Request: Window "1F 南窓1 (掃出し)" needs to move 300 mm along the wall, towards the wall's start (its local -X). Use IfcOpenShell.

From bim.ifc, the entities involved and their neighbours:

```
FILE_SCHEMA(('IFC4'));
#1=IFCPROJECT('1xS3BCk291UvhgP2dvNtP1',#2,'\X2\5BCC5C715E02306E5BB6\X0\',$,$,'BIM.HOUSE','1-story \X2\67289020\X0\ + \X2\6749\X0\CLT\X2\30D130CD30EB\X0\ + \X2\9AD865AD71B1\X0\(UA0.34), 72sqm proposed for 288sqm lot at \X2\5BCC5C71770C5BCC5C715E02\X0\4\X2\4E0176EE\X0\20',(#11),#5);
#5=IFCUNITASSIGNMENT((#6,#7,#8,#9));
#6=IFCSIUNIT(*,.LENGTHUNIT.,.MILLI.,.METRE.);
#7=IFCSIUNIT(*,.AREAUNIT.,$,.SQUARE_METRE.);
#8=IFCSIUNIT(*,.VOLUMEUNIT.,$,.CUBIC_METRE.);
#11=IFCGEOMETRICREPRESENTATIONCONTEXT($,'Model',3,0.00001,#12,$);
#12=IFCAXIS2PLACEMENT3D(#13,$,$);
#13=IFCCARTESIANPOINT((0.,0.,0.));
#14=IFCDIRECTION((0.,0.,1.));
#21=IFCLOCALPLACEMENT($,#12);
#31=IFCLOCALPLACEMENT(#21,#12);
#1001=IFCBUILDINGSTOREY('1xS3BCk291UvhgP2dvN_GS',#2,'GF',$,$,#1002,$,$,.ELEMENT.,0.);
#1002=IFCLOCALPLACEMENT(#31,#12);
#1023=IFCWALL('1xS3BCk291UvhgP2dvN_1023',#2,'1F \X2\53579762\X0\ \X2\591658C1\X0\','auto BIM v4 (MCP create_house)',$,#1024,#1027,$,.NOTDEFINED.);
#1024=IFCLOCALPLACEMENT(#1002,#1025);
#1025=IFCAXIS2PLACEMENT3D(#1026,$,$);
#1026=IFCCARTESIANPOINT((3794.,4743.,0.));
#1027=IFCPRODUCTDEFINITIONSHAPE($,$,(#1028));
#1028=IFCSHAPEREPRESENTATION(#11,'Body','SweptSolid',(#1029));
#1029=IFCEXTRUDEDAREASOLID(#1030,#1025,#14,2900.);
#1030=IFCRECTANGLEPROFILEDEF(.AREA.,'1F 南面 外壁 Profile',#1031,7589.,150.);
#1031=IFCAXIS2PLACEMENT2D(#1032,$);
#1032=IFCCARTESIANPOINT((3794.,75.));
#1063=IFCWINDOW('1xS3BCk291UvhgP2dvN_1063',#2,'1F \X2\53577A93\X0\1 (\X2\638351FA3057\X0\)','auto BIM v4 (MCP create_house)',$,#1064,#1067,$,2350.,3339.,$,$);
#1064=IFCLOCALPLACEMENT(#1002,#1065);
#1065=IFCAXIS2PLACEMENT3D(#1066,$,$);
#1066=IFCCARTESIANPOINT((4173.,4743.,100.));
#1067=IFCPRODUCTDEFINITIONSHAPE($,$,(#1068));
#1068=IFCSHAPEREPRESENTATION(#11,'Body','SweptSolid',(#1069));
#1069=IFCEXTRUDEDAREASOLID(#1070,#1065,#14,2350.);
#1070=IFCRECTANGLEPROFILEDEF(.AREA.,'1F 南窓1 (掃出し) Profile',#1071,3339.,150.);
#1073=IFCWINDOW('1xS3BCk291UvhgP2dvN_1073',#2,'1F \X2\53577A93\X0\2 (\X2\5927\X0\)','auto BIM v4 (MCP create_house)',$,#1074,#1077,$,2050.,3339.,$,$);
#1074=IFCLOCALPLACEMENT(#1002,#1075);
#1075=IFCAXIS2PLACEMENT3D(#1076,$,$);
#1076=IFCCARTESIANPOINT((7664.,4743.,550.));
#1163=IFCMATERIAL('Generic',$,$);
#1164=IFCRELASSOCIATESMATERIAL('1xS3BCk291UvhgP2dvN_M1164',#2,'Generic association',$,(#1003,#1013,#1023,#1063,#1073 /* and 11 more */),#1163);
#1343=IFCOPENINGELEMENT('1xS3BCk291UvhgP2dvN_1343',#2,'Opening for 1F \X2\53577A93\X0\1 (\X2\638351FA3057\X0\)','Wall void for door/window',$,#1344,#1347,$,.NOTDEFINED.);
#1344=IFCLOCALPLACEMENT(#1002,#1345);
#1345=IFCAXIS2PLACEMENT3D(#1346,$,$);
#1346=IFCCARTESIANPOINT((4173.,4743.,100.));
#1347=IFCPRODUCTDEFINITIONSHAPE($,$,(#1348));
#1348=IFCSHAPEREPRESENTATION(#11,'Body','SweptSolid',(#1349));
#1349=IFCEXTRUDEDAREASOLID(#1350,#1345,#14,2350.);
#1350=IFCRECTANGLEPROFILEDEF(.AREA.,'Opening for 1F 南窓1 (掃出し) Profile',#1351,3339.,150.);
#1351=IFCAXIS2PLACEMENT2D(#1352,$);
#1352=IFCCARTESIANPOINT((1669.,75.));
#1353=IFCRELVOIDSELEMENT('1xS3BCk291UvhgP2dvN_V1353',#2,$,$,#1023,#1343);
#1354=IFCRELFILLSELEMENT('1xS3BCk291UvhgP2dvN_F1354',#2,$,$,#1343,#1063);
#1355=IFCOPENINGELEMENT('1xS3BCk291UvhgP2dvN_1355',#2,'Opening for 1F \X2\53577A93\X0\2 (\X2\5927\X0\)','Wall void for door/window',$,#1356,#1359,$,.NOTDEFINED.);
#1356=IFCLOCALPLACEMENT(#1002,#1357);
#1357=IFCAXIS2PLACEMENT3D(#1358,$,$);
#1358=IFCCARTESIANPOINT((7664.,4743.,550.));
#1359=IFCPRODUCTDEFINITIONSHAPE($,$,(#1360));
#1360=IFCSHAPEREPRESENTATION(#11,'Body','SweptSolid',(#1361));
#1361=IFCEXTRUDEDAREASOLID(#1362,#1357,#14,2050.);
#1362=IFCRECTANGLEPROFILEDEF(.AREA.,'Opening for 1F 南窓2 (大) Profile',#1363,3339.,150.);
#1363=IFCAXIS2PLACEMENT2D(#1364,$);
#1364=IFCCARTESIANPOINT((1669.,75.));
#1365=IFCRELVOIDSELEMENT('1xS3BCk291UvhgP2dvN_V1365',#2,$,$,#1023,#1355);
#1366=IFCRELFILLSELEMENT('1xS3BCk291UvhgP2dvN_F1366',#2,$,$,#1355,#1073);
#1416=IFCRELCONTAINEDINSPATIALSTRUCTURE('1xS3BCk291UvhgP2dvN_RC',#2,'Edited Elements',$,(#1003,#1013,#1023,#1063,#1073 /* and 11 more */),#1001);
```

```python
import ifcopenshell
import ifcopenshell.api.geometry
import ifcopenshell.util.placement

model = ifcopenshell.open("bim.ifc")

window = model.by_id(1063)
opening = window.FillsVoids[0].RelatingOpeningElement
wall = opening.VoidsElements[0].RelatingBuildingElement

wall_matrix = ifcopenshell.util.placement.get_local_placement(wall.ObjectPlacement)
shift = wall_matrix[:3, 0] * -300.0
before = ifcopenshell.util.placement.get_local_placement(window.ObjectPlacement)[:3, 3].copy()

# The window is not placed relative to its opening, so move both.
for product in (opening, window):
    matrix = ifcopenshell.util.placement.get_local_placement(product.ObjectPlacement)
    matrix[:3, 3] += shift
    ifcopenshell.api.geometry.edit_object_placement(model, product=product, matrix=matrix, is_si=False)

after = ifcopenshell.util.placement.get_local_placement(window.ObjectPlacement)[:3, 3]
print("window moved by", (after - before).round(3) + 0.0)

model.write("bim-out.ifc")
```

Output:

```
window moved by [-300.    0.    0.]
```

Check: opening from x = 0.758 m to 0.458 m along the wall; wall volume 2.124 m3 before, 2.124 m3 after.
